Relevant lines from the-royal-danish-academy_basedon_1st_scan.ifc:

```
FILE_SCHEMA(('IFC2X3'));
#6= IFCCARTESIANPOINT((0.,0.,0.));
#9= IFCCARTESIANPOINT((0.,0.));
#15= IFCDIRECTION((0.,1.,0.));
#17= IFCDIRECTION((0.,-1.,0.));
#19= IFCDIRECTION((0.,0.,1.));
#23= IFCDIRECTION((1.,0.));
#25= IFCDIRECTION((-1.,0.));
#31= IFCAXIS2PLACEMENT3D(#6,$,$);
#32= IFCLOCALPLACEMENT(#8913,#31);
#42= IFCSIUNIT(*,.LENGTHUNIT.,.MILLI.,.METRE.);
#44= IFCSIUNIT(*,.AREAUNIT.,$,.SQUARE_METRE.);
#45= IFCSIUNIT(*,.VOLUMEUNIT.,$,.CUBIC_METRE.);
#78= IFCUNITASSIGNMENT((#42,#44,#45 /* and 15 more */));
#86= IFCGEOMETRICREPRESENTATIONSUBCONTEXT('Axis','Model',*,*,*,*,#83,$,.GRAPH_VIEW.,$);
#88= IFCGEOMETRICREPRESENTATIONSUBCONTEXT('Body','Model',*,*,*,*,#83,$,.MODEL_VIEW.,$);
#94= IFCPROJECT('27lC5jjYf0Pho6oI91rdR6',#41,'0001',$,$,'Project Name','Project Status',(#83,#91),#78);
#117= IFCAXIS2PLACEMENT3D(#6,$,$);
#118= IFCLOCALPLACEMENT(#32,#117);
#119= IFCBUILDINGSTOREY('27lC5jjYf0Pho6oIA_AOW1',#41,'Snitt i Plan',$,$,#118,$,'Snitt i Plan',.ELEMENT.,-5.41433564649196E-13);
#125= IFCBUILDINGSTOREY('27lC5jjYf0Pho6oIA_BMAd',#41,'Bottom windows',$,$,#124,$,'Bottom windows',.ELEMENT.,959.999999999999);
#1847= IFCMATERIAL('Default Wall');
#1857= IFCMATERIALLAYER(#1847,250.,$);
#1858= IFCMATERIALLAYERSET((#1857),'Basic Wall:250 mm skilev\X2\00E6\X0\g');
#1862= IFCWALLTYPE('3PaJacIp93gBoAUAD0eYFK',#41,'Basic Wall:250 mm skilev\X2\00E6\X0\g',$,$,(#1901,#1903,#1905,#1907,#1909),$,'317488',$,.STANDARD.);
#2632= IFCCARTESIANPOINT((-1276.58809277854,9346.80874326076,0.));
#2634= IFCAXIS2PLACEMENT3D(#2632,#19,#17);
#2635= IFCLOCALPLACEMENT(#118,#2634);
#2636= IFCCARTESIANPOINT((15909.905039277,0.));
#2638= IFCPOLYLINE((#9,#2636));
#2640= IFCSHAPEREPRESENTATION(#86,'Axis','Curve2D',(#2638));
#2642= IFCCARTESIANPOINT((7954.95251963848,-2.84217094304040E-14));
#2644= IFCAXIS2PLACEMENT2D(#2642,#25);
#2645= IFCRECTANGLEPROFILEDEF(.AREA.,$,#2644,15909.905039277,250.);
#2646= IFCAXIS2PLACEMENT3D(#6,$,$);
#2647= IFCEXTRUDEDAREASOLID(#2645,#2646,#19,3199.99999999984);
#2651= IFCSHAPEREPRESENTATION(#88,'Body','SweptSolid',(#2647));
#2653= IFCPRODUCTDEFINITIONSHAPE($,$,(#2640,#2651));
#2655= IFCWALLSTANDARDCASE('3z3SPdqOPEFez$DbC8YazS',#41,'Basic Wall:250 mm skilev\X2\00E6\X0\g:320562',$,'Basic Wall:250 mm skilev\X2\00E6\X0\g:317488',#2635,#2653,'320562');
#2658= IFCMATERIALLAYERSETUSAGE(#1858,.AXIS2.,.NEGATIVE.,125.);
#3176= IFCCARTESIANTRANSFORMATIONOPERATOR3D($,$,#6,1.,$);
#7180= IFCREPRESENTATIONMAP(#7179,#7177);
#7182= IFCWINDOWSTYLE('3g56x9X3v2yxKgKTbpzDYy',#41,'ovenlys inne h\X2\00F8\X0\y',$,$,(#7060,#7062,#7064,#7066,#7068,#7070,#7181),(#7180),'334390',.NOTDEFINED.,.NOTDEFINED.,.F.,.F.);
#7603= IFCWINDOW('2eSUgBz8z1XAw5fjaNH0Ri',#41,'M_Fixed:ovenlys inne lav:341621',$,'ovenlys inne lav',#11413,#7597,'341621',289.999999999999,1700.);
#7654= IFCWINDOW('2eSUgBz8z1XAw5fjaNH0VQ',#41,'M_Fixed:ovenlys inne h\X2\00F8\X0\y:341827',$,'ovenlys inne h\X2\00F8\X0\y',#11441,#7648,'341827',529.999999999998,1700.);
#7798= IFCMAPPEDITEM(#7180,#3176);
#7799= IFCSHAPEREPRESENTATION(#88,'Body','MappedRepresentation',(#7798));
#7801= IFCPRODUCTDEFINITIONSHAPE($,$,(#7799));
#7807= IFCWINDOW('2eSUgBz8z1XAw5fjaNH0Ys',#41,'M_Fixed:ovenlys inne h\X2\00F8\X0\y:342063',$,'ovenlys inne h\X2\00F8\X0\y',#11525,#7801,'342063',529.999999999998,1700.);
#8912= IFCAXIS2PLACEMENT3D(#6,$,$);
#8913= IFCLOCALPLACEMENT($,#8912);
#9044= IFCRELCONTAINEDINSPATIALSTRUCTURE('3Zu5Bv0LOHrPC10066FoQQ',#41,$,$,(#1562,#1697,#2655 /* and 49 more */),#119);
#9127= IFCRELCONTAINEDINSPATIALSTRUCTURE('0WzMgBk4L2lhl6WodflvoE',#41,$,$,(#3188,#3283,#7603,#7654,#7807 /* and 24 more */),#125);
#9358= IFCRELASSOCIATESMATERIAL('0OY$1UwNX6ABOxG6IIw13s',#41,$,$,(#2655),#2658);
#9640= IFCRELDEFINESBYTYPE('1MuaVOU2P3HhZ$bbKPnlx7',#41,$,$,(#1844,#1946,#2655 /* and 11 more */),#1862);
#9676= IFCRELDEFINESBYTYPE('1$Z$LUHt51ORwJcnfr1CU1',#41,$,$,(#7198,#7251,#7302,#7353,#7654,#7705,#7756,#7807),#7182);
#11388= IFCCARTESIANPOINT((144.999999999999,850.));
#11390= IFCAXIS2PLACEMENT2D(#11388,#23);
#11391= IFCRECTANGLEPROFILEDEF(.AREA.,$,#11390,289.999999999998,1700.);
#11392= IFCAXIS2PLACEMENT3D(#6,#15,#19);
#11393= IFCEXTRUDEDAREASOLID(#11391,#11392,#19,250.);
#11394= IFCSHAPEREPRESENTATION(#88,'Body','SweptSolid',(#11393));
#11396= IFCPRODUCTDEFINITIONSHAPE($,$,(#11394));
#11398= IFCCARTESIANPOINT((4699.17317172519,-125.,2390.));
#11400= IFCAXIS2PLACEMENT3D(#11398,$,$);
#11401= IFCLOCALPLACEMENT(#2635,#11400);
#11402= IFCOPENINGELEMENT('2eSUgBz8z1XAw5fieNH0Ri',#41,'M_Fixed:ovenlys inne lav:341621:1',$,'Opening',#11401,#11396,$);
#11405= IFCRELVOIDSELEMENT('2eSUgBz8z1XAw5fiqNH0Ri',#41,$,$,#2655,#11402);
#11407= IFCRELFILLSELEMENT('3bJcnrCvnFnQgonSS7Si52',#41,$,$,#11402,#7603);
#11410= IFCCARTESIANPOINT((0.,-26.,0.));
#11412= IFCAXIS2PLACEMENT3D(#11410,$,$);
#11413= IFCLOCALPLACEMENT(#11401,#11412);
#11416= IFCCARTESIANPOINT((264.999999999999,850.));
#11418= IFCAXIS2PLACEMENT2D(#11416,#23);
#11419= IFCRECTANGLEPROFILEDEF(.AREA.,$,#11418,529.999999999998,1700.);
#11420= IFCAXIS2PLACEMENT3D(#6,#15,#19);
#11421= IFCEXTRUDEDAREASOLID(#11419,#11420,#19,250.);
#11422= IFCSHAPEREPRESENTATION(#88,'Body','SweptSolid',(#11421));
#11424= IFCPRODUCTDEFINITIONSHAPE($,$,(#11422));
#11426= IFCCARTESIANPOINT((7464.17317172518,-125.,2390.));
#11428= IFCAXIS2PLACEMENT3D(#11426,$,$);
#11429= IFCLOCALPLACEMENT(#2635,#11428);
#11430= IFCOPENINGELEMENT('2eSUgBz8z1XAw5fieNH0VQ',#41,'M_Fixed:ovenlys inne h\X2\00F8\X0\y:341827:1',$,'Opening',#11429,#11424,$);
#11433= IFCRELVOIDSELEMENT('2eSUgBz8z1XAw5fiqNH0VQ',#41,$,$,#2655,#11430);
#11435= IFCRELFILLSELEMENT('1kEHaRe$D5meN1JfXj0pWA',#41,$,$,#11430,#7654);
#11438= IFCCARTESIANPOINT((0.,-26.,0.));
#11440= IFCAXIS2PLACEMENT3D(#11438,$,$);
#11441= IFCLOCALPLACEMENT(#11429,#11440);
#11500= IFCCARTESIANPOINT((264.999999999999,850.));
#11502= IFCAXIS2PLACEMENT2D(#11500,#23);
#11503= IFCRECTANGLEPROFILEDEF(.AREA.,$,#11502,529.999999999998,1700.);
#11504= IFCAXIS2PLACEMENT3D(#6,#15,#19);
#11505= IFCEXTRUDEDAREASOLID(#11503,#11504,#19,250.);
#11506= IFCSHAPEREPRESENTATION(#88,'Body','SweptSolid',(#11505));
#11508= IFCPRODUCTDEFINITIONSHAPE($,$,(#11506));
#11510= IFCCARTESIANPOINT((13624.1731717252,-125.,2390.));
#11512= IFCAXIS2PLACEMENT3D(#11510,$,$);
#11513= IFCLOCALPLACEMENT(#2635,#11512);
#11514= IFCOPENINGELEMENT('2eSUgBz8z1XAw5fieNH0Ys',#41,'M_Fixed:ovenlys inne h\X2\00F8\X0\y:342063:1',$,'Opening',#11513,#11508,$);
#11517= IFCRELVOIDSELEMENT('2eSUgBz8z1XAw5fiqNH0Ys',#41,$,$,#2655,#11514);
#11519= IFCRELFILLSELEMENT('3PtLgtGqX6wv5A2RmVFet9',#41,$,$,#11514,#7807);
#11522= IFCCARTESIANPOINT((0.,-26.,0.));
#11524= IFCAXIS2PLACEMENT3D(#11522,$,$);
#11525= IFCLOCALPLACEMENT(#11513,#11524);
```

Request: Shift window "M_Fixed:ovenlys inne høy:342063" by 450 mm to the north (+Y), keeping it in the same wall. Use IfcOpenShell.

```python
import ifcopenshell
import ifcopenshell.api.geometry
import ifcopenshell.util.placement
import ifcopenshell.util.unit

model = ifcopenshell.open("the-royal-danish-academy_basedon_1st_scan.ifc")
unit_scale = ifcopenshell.util.unit.calculate_unit_scale(model)

window = model.by_id(7807)
opening = window.FillsVoids[0].RelatingOpeningElement
wall = opening.VoidsElements[0].RelatingBuildingElement

wall_matrix = ifcopenshell.util.placement.get_local_placement(wall.ObjectPlacement)
shift = wall_matrix[:3, 0] * -0.45 / unit_scale
before = ifcopenshell.util.placement.get_local_placement(window.ObjectPlacement)[:3, 3].copy()

# The window is placed relative to its opening, so it follows when the opening moves.
matrix = ifcopenshell.util.placement.get_local_placement(opening.ObjectPlacement)
matrix[:3, 3] += shift
ifcopenshell.api.geometry.edit_object_placement(
    model, product=opening, matrix=matrix, is_si=False, should_transform_children=True
)

after = ifcopenshell.util.placement.get_local_placement(window.ObjectPlacement)[:3, 3]
print("window moved by", (after - before).round(3) + 0.0)

model.write("the-royal-danish-academy_basedon_1st_scan-out.ifc")
```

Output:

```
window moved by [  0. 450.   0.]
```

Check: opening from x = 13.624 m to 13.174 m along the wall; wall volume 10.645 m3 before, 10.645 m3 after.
